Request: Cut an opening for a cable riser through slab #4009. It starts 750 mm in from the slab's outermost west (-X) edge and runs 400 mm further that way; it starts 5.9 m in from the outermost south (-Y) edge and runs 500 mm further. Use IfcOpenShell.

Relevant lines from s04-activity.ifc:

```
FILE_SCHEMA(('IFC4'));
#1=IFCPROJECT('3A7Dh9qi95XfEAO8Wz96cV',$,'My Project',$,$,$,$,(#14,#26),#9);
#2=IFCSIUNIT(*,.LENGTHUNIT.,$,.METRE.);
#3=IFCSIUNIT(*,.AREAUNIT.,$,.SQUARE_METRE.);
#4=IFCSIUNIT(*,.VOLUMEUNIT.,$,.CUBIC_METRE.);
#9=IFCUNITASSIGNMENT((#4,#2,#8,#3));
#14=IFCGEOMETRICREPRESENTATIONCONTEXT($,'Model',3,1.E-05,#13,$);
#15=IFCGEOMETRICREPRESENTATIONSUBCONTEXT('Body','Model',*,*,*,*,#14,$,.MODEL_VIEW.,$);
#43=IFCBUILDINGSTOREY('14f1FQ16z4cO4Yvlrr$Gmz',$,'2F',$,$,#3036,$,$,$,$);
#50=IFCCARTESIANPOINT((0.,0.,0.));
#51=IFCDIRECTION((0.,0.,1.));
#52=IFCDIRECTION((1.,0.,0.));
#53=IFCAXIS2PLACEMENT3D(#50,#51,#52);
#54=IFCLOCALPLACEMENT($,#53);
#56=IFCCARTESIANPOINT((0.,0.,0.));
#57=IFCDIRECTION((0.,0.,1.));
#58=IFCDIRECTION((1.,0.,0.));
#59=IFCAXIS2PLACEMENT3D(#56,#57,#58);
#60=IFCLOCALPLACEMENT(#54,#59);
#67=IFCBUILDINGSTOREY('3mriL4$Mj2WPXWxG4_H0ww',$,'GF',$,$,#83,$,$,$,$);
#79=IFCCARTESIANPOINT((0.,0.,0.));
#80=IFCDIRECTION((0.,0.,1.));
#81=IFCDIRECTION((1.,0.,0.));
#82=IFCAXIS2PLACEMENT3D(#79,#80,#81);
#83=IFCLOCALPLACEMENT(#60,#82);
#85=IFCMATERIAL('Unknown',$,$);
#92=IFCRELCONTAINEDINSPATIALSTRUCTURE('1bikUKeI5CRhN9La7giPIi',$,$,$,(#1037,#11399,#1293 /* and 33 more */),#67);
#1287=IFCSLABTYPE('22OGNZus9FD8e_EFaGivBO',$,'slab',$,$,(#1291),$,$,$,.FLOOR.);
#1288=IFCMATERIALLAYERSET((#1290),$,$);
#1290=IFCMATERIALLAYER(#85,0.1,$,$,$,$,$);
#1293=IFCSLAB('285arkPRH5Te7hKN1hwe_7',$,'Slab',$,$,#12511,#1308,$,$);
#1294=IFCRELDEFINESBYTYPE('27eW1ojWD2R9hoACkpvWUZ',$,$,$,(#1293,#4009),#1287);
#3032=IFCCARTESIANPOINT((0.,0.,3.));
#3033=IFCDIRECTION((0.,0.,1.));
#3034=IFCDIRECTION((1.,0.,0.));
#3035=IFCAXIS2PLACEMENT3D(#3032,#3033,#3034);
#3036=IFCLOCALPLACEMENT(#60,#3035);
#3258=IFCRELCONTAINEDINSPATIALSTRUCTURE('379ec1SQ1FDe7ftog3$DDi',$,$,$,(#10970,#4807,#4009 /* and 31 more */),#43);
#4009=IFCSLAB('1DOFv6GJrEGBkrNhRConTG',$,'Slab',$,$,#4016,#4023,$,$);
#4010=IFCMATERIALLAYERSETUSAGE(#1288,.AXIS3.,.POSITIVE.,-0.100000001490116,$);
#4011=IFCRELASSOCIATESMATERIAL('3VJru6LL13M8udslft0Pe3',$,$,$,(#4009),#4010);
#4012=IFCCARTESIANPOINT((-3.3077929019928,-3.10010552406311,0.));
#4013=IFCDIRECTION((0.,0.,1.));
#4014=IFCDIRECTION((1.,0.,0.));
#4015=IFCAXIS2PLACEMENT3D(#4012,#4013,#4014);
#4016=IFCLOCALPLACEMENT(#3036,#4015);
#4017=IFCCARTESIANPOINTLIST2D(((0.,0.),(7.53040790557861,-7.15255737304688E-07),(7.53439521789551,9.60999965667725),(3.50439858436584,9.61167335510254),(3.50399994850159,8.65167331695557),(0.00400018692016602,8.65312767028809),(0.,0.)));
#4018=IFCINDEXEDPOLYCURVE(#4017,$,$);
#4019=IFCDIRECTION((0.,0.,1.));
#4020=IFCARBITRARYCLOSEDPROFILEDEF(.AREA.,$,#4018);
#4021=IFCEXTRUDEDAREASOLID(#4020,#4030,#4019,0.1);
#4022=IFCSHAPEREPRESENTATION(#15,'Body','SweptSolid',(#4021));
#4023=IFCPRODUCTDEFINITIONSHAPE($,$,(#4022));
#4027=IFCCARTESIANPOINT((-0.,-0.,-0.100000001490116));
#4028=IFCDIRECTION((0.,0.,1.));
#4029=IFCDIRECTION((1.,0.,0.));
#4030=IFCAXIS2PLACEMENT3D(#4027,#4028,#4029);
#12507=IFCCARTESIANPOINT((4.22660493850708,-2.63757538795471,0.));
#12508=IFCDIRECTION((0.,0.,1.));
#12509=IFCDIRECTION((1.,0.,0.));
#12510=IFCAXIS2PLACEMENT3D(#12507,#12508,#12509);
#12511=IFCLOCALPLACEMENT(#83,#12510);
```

```python
import numpy as np
import ifcopenshell
import ifcopenshell.api.feature
import ifcopenshell.api.geometry
import ifcopenshell.api.root
import ifcopenshell.geom
import ifcopenshell.util.placement
import ifcopenshell.util.representation
import ifcopenshell.util.shape
import ifcopenshell.util.unit

model = ifcopenshell.open("s04-activity.ifc")
unit_scale = ifcopenshell.util.unit.calculate_unit_scale(model)
settings = ifcopenshell.geom.settings()


def volume(element):
    """Net volume in cubic metres, openings subtracted."""
    shape = ifcopenshell.geom.create_shape(settings, element)
    return ifcopenshell.util.shape.get_volume(shape.geometry)


slab = model.by_guid("1DOFv6GJrEGBkrNhRConTG")
before = volume(slab)

# Extent in the slab's own axes, in metres. The edges named are its -X and -Y sides.
slab_shape = ifcopenshell.geom.create_shape(settings, slab)
vertices = ifcopenshell.util.shape.get_vertices(slab_shape.geometry)
x_min, y_min, bottom = vertices.min(axis=0)
top = vertices[:, 2].max()

opening = ifcopenshell.api.root.create_entity(model, ifc_class="IfcOpeningElement", name="Cable riser opening", predefined_type="OPENING")
context = ifcopenshell.util.representation.get_context(model, "Model", "Body", "MODEL_VIEW")
width, depth = 0.4, 0.5
outline = [(0.0, 0.0), (width, 0.0), (width, depth), (0.0, depth), (0.0, 0.0)]
# Overshoot both faces by 50 mm so the cut is clean.
shape = ifcopenshell.api.geometry.add_slab_representation(
    model, context=context, depth=top - bottom + 0.1, polyline=outline
)
ifcopenshell.api.geometry.assign_representation(model, product=opening, representation=shape)

matrix = ifcopenshell.util.placement.get_local_placement(slab.ObjectPlacement)
matrix[:, 3] = matrix @ np.append(np.array([x_min + 0.75, y_min + 5.9, bottom - 0.05]) / unit_scale, 1.0)
ifcopenshell.api.geometry.edit_object_placement(model, product=opening, matrix=matrix, is_si=False)
ifcopenshell.api.feature.add_feature(model, feature=opening, element=slab)

after = volume(slab)

print(f"slab volume {before:.3f} -> {after:.3f} m3")

model.write("s04-activity_v2.ifc")
```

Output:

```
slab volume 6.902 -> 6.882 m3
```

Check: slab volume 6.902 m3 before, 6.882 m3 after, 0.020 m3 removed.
